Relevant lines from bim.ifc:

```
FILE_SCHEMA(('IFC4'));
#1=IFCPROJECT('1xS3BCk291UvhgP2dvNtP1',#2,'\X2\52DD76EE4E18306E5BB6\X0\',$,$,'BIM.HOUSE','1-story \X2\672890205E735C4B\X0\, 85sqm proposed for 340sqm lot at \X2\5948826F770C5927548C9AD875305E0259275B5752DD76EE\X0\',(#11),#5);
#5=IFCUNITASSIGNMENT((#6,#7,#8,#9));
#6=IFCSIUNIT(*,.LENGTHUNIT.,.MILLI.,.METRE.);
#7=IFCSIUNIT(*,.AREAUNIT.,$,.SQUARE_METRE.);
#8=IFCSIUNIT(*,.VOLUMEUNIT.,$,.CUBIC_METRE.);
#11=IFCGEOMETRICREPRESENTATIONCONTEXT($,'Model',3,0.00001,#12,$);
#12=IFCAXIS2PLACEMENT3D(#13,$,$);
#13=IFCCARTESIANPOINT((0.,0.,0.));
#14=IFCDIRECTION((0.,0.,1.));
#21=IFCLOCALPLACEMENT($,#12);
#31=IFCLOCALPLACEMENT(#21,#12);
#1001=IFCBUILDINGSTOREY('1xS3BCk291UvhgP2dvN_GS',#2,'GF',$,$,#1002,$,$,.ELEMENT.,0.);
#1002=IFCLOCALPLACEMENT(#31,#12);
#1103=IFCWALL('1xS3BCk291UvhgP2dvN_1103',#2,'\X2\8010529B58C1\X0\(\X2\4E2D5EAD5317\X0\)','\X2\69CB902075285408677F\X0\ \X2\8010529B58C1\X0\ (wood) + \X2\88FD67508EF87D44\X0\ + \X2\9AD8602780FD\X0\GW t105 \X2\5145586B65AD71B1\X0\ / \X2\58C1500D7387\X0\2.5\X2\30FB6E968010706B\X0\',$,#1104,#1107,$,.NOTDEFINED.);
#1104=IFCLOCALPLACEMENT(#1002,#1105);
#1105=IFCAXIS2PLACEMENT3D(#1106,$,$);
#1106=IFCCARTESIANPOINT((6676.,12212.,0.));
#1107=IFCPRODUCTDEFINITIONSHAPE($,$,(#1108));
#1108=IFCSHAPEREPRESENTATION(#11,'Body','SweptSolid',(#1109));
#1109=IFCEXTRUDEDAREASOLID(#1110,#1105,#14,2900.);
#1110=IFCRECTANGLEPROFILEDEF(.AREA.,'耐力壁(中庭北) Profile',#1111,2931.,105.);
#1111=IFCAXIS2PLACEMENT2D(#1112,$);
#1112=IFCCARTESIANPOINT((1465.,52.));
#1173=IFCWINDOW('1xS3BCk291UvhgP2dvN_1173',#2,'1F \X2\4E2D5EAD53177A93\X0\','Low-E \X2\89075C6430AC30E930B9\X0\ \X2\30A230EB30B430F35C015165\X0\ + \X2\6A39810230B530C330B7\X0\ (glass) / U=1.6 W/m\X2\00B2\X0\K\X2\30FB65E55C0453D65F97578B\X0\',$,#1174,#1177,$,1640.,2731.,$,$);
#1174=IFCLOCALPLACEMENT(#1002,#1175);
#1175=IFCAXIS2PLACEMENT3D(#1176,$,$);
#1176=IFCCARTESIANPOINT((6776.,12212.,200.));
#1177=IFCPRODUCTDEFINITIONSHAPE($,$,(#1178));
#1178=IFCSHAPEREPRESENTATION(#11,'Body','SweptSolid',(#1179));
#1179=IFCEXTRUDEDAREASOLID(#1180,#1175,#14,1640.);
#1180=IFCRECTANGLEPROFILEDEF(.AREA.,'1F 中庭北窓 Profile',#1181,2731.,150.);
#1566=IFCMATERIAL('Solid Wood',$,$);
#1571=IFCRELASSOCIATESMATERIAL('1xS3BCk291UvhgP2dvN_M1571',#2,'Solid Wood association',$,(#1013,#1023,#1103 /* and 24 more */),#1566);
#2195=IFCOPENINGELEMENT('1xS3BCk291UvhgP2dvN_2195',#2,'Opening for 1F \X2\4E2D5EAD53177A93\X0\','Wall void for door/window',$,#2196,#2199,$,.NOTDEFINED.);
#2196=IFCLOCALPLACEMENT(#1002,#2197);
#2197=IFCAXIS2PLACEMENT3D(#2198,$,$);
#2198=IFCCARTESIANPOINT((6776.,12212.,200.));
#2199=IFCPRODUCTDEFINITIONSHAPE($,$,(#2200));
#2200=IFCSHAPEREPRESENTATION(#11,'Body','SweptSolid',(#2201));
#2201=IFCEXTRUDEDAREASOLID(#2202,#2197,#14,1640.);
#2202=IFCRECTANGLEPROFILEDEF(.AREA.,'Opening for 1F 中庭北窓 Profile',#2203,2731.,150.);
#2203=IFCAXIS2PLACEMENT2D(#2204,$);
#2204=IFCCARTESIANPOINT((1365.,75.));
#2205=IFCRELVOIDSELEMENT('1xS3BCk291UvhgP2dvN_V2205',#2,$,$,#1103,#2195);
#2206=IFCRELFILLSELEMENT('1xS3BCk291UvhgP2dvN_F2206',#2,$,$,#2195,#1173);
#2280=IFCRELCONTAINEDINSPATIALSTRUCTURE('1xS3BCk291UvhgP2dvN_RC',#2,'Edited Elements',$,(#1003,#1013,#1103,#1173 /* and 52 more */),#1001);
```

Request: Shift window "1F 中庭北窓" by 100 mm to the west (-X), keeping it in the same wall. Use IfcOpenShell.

```python
import ifcopenshell
import ifcopenshell.api.geometry
import ifcopenshell.util.placement

model = ifcopenshell.open("bim.ifc")

window = model.by_guid("1xS3BCk291UvhgP2dvN_1173")
opening = window.FillsVoids[0].RelatingOpeningElement
wall = opening.VoidsElements[0].RelatingBuildingElement

wall_matrix = ifcopenshell.util.placement.get_local_placement(wall.ObjectPlacement)
shift = wall_matrix[:3, 0] * -100.0
before = ifcopenshell.util.placement.get_local_placement(window.ObjectPlacement)[:3, 3].copy()

# The window is not placed relative to its opening, so move both.
for product in (opening, window):
    matrix = ifcopenshell.util.placement.get_local_placement(product.ObjectPlacement)
    matrix[:3, 3] += shift
    ifcopenshell.api.geometry.edit_object_placement(model, product=product, matrix=matrix, is_si=False)

after = ifcopenshell.util.placement.get_local_placement(window.ObjectPlacement)[:3, 3]
print("window moved by", (after - before).round(3) + 0.0)

model.write("bim-out.ifc")
```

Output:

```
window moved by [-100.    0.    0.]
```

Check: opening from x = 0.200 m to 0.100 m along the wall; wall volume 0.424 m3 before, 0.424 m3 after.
